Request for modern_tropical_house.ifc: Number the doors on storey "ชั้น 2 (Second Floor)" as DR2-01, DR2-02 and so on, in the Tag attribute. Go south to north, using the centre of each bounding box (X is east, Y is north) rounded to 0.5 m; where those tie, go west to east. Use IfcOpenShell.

First a look at what the model holds.

```python
import ifcopenshell
import ifcopenshell.util.element
import ifcopenshell.util.placement

model = ifcopenshell.open("modern_tropical_house.ifc")
print(model.schema)
storey = next(s for s in model.by_type("IfcBuildingStorey") if s.Name == "ชั้น 2 (Second Floor)")
doors = [e for e in ifcopenshell.util.element.get_decomposition(storey) if e.is_a("IfcDoor")]
for e in sorted(doors, key=lambda e: e.id()):
    origin = ifcopenshell.util.placement.get_local_placement(e.ObjectPlacement)[:3, 3]
    print(e.id(), e.Tag, e.Name, origin.round(2) + 0.0, sep=" | ")
```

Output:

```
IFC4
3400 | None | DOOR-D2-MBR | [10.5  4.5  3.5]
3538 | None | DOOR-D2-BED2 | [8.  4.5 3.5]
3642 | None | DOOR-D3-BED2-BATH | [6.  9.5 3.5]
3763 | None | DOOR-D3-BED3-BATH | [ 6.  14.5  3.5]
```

```python
import ifcopenshell
import ifcopenshell.geom
import ifcopenshell.util.element
import ifcopenshell.util.shape

model = ifcopenshell.open("modern_tropical_house.ifc")
settings = ifcopenshell.geom.settings()
settings.set("use-world-coords", True)


def centre(element):
    shape = ifcopenshell.geom.create_shape(settings, element)
    return ifcopenshell.util.shape.get_bbox_centroid(shape.geometry)


storey = next(s for s in model.by_type("IfcBuildingStorey") if s.Name == "ชั้น 2 (Second Floor)")
doors = [e for e in ifcopenshell.util.element.get_decomposition(storey) if e.is_a("IfcDoor")]

# Insertion points can sit at a corner or the storey origin, so sort by the geometry (in metres).
centres = {e: centre(e) for e in doors}
doors.sort(key=lambda e: (round(centres[e][1] / 0.5), centres[e][0]))

for i, e in enumerate(doors, start=1):
    number = f"DR2-{i:02d}"
    e.Tag = number
    print(e.id(), number)

model.write("modern_tropical_house_updated.ifc")
```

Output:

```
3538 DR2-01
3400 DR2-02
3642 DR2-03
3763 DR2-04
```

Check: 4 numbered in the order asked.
